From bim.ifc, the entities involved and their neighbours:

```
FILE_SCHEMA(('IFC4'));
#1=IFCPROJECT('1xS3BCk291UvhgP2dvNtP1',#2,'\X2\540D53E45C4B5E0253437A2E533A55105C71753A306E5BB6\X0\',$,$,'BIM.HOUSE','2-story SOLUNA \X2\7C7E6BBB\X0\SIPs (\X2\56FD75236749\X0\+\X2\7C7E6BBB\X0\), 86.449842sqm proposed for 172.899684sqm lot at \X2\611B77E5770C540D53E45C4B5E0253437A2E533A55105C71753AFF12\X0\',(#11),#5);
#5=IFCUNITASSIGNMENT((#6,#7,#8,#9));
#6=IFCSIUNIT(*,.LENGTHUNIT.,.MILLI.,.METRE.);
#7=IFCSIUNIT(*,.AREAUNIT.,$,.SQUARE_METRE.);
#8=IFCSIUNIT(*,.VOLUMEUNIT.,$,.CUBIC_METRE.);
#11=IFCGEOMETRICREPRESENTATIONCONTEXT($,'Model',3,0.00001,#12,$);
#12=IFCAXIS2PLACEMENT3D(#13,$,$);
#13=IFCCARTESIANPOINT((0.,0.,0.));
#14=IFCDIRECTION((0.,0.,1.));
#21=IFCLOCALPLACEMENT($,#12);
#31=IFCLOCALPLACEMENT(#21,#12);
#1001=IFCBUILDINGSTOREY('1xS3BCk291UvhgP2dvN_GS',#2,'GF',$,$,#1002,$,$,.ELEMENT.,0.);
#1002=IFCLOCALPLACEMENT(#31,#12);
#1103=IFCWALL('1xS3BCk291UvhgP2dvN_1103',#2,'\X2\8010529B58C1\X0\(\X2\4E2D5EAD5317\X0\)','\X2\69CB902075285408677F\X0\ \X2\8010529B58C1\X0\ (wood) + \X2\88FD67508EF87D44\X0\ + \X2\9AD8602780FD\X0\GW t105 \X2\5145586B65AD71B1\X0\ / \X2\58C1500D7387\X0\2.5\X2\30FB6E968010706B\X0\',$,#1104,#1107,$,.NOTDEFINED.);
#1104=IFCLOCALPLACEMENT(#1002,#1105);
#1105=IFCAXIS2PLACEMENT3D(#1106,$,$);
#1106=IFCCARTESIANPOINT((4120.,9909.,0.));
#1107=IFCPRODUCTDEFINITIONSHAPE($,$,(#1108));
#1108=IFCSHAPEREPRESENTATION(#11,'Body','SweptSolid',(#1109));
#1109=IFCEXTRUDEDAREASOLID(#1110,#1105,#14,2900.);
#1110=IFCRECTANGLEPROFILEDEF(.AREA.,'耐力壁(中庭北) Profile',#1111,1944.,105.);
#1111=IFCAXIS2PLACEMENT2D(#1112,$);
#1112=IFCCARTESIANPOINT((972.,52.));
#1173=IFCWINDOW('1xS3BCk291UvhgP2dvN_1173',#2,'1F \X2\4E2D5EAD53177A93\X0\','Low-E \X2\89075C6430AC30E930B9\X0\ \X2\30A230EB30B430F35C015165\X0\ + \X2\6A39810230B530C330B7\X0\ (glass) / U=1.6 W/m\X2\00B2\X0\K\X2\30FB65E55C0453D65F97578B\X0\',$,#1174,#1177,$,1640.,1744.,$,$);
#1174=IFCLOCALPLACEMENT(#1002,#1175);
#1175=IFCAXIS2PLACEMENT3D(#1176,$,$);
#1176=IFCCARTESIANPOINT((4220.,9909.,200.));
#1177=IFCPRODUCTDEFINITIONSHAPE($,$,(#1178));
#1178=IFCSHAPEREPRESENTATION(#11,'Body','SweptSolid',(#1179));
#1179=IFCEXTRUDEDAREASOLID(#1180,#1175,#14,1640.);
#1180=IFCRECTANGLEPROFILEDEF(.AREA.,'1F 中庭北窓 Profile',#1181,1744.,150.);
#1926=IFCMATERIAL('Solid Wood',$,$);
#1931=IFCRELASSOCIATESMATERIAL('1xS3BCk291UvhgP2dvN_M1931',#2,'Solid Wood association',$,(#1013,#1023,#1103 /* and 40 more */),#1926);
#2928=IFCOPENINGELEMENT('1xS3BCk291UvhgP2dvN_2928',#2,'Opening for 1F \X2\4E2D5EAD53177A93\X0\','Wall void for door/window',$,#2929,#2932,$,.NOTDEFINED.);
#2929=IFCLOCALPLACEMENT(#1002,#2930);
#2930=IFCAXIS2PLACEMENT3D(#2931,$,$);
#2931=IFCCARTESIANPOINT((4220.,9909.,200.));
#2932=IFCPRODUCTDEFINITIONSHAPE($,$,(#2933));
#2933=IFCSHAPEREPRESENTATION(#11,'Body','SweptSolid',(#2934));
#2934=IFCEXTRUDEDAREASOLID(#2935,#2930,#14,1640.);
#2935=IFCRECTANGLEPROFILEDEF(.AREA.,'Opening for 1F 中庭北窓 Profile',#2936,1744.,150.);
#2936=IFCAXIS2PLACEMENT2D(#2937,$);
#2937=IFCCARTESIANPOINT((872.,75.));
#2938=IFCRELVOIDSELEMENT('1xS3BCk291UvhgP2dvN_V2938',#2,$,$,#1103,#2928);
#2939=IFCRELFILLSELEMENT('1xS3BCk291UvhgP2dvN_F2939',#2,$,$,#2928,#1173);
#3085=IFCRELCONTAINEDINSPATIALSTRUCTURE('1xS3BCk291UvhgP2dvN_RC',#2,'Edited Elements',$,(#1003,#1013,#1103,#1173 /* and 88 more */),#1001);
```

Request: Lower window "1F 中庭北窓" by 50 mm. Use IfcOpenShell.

```python
import numpy as np
import ifcopenshell
import ifcopenshell.api.geometry
import ifcopenshell.util.placement
import ifcopenshell.util.unit

model = ifcopenshell.open("bim.ifc")
unit_scale = ifcopenshell.util.unit.calculate_unit_scale(model)

window = model.by_guid("1xS3BCk291UvhgP2dvN_1173")
opening = window.FillsVoids[0].RelatingOpeningElement
dz = -0.05 / unit_scale

shift = np.array([0.0, 0.0, dz])
# The window is not placed relative to its opening, so move both.
for product in (opening, window):
    matrix = ifcopenshell.util.placement.get_local_placement(product.ObjectPlacement)
    matrix[:3, 3] += shift
    ifcopenshell.api.geometry.edit_object_placement(model, product=product, matrix=matrix, is_si=False)

print(f"moved by {dz * unit_scale:+.3f} m")

model.write("bim_rev.ifc")
```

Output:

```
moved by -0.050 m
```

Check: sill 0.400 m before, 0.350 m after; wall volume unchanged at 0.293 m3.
